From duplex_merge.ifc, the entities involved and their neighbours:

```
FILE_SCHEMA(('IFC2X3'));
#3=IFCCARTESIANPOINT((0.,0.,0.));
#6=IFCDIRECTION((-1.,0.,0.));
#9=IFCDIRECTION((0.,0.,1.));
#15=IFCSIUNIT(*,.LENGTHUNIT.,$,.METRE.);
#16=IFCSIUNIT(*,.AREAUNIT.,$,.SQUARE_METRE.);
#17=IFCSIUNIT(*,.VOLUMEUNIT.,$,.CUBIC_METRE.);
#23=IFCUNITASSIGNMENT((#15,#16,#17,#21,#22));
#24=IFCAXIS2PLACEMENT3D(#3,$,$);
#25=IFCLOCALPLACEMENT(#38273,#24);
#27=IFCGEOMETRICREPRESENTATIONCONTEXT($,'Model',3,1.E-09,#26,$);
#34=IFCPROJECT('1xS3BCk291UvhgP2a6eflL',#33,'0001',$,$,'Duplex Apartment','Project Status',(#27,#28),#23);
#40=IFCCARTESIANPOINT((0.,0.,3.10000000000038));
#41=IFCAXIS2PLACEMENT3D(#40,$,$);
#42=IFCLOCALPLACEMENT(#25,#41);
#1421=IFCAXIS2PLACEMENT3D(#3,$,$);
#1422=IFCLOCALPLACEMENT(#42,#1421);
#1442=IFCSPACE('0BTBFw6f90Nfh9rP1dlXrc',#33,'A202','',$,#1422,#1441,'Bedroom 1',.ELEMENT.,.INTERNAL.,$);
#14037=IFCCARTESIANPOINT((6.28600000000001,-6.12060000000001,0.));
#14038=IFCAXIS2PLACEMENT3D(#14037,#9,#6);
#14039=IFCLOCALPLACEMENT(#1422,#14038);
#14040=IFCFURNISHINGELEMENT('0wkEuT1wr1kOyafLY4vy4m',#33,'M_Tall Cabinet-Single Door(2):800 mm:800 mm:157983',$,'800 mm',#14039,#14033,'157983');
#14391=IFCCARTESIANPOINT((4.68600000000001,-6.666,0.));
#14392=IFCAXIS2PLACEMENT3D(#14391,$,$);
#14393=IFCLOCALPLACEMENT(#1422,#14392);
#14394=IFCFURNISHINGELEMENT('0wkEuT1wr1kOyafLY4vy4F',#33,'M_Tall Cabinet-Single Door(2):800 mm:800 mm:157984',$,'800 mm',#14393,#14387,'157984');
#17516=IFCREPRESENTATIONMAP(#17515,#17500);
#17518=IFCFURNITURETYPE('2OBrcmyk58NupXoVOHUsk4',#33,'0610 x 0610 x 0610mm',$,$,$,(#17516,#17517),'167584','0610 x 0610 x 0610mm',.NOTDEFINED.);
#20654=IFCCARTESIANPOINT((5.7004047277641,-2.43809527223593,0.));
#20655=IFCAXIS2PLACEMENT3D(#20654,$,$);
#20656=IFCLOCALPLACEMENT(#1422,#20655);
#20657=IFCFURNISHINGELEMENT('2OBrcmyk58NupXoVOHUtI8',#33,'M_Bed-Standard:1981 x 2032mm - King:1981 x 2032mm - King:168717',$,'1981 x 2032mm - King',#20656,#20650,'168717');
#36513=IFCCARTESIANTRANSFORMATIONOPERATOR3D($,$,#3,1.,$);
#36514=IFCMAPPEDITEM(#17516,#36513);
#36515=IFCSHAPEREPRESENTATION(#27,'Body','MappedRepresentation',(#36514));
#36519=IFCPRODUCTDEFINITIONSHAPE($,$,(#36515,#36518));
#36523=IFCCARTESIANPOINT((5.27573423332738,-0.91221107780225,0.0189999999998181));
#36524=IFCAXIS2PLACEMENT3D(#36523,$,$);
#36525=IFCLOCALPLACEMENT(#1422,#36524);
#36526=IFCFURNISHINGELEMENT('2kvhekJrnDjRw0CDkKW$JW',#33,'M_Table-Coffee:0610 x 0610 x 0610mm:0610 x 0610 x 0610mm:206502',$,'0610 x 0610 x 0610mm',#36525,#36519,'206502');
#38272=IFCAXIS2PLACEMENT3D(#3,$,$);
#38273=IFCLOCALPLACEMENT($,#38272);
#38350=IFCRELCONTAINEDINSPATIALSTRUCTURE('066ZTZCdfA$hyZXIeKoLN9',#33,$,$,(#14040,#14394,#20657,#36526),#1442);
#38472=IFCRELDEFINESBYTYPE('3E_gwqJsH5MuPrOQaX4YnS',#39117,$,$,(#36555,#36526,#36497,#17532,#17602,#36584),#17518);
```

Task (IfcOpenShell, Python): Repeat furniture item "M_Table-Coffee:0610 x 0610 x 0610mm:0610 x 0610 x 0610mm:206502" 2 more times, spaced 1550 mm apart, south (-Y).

```python
import numpy as np
import ifcopenshell
import ifcopenshell.api.geometry
import ifcopenshell.api.root
import ifcopenshell.util.element
import ifcopenshell.util.placement
import ifcopenshell.util.unit

model = ifcopenshell.open("duplex_merge.ifc")
unit_scale = ifcopenshell.util.unit.calculate_unit_scale(model)


def reuse_history(source, copy):
    """copy_class also copies each property set's owner history, people and application; keep the originals."""
    for rel in copy.IsDefinedBy:
        if rel.is_a("IfcRelDefinesByProperties") and (history := rel.RelatingPropertyDefinition.OwnerHistory):
            rel.RelatingPropertyDefinition.OwnerHistory = source.OwnerHistory
            ifcopenshell.util.element.remove_deep2(model, history)


source = model.by_guid("2kvhekJrnDjRw0CDkKW$JW")
base = ifcopenshell.util.placement.get_local_placement(source.ObjectPlacement)
step = np.array([0.0, -1.0, 0.0]) * 1.55 / unit_scale

for i in range(1, 3):
    copy = ifcopenshell.api.root.copy_class(model, product=source)
    copy.Representation = ifcopenshell.util.element.copy_deep(
        model, source.Representation, exclude=["IfcGeometricRepresentationContext", "IfcRepresentationMap"]
    )
    copy.Name = "M_Table-Coffee:0610 x 0610 x 0610mm:0610 x 0610 x 0610mm"
    copy.Tag = None
    reuse_history(source, copy)
    matrix = base.copy()
    matrix[:3, 3] += i * step
    print("added at", matrix[:3, 3].round(3) + 0.0)
    ifcopenshell.api.geometry.edit_object_placement(model, product=copy, matrix=matrix, is_si=False)

model.write("duplex_merge_v2.ifc")
```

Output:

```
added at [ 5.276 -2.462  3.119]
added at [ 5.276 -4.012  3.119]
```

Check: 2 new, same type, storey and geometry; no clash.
